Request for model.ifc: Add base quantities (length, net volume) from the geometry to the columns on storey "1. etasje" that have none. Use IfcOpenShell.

First a look at what the model holds.

```python
import ifcopenshell
import ifcopenshell.util.element
import ifcopenshell.util.unit

model = ifcopenshell.open("model.ifc")
print(model.schema)
for unit_type in ("LENGTHUNIT", "AREAUNIT", "VOLUMEUNIT"):
    print(unit_type, ifcopenshell.util.unit.calculate_unit_scale(model, unit_type))
storey = next(s for s in model.by_type("IfcBuildingStorey") if s.Name == "1. etasje")
columns = [e for e in ifcopenshell.util.element.get_decomposition(storey) if e.is_a("IfcColumn")]
for e in sorted(columns, key=lambda e: e.id()):
    print(e.id(), e.is_a(), e.Name, list(ifcopenshell.util.element.get_psets(e, qtos_only=True)), sep=" | ")
```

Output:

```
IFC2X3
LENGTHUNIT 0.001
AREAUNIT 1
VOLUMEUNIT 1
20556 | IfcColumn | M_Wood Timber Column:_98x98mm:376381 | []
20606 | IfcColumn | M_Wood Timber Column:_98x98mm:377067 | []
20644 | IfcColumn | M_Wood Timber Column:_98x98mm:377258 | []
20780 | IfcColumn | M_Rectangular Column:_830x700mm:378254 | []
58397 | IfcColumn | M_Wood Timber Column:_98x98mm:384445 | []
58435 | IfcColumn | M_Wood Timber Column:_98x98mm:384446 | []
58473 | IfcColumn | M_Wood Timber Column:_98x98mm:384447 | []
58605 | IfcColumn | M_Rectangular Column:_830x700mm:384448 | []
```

```python
import ifcopenshell
import ifcopenshell.api.pset
import ifcopenshell.geom
import ifcopenshell.util.element
import ifcopenshell.util.shape
import ifcopenshell.util.unit

model = ifcopenshell.open("model.ifc")
unit_scale = ifcopenshell.util.unit.calculate_unit_scale(model)
volume_scale = ifcopenshell.util.unit.calculate_unit_scale(model, "VOLUMEUNIT")
settings = ifcopenshell.geom.settings()

storey = next(s for s in model.by_type("IfcBuildingStorey") if s.Name == "1. etasje")
columns = [e for e in ifcopenshell.util.element.get_decomposition(storey) if e.is_a("IfcColumn")]

for e in sorted(columns, key=lambda e: e.id()):
    if ifcopenshell.util.element.get_psets(e, qtos_only=True, should_inherit=False):
        continue
    # Geometry comes back in metres, in the element's own axes.
    shape = ifcopenshell.geom.create_shape(settings, e)
    values = {
        "Length": ifcopenshell.util.shape.get_z(shape.geometry) / unit_scale,
        "NetVolume": ifcopenshell.util.shape.get_volume(shape.geometry) / volume_scale,
    }
    qto = ifcopenshell.api.pset.add_qto(model, product=e, name="BaseQuantities")
    ifcopenshell.api.pset.edit_qto(model, qto=qto, properties=values)
    print(e.id(), {k: round(v, 3) for k, v in values.items()})

model.write("model_edited.ifc")
```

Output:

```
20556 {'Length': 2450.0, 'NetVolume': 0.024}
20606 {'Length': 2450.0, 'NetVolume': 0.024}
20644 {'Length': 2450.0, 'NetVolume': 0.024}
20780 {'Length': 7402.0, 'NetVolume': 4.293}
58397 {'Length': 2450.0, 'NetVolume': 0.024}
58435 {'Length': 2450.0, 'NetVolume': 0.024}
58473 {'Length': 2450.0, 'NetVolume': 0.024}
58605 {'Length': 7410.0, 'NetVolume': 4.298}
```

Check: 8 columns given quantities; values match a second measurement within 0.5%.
